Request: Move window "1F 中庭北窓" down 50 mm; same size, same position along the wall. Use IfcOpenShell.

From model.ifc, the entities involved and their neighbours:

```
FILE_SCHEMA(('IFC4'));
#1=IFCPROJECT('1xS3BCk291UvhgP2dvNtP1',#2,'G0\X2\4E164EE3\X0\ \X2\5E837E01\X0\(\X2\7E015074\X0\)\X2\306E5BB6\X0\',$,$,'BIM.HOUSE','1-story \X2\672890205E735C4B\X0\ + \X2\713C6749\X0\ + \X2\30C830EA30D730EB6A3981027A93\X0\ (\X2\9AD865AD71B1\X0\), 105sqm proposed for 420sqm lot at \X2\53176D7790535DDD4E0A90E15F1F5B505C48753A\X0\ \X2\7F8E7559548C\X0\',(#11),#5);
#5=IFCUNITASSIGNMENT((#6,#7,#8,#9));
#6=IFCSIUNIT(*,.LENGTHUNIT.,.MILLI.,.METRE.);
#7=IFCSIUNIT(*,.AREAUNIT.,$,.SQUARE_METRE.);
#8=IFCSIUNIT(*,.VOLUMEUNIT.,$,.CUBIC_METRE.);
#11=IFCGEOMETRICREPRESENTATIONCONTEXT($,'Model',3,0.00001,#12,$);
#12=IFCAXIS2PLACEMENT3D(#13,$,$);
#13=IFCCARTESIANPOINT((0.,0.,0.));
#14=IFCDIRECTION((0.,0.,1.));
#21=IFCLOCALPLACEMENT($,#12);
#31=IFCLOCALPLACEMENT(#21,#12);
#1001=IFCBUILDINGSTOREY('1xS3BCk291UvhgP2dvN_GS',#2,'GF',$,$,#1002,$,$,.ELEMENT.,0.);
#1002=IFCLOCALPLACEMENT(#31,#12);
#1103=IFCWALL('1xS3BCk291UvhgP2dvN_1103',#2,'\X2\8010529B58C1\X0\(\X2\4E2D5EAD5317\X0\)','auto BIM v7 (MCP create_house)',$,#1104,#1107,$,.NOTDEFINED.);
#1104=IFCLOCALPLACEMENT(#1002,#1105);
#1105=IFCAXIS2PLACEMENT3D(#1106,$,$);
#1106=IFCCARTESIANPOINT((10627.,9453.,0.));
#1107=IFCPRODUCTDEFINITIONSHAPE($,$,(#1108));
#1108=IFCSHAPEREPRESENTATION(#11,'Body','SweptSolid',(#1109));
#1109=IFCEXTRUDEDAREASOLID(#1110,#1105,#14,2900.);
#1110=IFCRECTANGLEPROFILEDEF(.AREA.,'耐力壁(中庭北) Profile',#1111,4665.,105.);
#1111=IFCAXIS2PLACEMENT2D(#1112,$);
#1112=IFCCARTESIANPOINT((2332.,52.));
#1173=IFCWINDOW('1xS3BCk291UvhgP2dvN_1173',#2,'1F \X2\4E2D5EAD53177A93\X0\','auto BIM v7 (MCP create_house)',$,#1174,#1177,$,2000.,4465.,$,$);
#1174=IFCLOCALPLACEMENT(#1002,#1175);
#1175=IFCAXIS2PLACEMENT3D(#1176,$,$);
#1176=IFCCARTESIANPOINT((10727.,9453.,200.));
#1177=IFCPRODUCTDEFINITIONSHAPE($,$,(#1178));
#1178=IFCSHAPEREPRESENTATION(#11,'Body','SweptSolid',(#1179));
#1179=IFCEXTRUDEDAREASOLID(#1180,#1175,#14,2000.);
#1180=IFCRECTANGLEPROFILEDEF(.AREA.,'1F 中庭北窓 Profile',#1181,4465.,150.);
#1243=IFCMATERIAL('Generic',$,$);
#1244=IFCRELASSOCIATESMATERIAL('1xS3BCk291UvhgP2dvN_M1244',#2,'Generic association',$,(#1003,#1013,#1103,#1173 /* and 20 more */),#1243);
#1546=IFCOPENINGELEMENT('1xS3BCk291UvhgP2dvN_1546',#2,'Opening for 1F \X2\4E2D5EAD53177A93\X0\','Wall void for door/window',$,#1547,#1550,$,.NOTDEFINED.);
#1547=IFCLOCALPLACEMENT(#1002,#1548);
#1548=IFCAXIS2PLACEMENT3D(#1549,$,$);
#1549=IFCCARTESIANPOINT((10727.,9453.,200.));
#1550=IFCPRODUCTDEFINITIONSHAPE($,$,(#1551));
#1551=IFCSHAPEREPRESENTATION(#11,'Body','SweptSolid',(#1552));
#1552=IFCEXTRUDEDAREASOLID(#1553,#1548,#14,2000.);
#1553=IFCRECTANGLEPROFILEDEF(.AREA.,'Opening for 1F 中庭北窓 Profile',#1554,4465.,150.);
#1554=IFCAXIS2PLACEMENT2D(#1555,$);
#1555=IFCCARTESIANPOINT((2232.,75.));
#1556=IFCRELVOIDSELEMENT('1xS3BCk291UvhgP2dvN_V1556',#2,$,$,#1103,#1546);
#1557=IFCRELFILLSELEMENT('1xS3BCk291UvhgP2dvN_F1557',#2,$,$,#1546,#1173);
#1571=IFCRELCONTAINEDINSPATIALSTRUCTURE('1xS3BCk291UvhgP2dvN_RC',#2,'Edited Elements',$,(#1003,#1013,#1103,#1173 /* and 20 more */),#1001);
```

```python
import numpy as np
import ifcopenshell
import ifcopenshell.api.geometry
import ifcopenshell.util.placement
import ifcopenshell.util.unit

model = ifcopenshell.open("model.ifc")
unit_scale = ifcopenshell.util.unit.calculate_unit_scale(model)

window = model.by_guid("1xS3BCk291UvhgP2dvN_1173")
opening = window.FillsVoids[0].RelatingOpeningElement
dz = -0.05 / unit_scale

shift = np.array([0.0, 0.0, dz])
# The window is not placed relative to its opening, so move both.
for product in (opening, window):
    matrix = ifcopenshell.util.placement.get_local_placement(product.ObjectPlacement)
    matrix[:3, 3] += shift
    ifcopenshell.api.geometry.edit_object_placement(model, product=product, matrix=matrix, is_si=False)

print(f"moved by {dz * unit_scale:+.3f} m")

model.write("model_edited.ifc")
```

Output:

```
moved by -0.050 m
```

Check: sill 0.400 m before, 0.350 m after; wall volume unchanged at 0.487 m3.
